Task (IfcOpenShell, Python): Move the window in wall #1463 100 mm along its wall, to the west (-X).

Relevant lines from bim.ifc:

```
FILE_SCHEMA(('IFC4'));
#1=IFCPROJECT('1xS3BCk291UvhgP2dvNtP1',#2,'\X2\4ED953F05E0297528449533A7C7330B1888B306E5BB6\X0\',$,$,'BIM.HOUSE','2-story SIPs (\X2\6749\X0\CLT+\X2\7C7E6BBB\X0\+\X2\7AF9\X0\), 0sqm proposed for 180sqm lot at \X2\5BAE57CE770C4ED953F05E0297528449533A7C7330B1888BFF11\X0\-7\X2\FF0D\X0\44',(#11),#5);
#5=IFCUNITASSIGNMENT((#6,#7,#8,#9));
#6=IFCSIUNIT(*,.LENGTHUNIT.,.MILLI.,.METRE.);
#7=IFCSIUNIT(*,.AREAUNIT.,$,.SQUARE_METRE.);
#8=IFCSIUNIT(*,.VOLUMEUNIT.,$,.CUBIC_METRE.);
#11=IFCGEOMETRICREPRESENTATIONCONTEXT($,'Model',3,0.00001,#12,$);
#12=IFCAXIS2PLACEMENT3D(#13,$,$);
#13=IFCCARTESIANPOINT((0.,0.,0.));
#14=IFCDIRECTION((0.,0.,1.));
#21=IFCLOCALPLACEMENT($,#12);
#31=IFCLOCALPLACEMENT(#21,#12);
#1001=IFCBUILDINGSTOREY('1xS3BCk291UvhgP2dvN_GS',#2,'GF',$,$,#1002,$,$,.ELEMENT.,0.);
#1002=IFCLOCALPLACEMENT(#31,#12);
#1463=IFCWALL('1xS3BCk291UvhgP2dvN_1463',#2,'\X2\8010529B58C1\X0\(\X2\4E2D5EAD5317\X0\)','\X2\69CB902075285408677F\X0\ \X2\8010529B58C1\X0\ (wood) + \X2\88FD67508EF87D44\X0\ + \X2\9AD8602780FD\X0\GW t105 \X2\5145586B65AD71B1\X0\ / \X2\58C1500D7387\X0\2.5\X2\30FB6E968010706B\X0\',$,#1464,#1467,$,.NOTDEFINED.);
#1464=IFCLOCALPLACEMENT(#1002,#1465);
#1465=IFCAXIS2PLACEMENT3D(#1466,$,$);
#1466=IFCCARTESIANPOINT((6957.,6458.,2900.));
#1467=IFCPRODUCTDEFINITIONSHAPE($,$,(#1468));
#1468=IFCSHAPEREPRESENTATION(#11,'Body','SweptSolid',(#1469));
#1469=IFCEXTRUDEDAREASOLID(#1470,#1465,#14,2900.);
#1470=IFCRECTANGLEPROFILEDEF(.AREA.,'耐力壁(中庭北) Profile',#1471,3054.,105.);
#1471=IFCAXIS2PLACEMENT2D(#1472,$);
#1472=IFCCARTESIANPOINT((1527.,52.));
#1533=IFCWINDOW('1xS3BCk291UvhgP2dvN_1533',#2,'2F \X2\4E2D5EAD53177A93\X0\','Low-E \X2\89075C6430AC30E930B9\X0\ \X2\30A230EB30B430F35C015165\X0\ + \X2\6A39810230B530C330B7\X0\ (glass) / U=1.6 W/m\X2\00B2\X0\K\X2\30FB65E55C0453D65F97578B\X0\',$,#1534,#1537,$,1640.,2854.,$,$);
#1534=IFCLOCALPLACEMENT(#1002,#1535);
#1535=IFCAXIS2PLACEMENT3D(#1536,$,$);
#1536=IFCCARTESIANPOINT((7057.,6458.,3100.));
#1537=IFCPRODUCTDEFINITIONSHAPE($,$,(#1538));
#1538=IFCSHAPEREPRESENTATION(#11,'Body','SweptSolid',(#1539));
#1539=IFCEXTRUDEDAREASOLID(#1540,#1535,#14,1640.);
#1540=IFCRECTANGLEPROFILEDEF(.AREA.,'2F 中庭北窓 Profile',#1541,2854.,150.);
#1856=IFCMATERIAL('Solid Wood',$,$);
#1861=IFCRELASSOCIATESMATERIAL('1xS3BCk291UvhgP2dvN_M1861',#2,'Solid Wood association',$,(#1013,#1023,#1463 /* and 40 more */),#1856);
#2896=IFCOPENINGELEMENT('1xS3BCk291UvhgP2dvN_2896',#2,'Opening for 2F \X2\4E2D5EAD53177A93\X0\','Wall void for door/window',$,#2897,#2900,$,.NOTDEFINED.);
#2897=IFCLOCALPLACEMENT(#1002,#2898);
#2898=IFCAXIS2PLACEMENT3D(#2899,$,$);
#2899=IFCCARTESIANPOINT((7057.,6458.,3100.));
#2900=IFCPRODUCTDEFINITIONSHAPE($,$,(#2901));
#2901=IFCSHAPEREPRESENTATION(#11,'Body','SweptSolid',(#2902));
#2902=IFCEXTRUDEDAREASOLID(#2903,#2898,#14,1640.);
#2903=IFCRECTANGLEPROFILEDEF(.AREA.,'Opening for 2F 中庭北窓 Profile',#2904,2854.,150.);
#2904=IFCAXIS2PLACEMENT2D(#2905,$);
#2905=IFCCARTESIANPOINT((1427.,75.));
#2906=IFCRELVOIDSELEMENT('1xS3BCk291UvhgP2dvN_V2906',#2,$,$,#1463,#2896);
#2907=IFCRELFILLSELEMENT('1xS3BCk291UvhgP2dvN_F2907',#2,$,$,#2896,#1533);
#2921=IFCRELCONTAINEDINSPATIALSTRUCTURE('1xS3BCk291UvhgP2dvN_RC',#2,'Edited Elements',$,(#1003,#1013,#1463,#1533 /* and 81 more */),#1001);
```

```python
import ifcopenshell
import ifcopenshell.api.geometry
import ifcopenshell.util.placement
import ifcopenshell.util.unit

model = ifcopenshell.open("bim.ifc")
unit_scale = ifcopenshell.util.unit.calculate_unit_scale(model)

window = model.by_guid("1xS3BCk291UvhgP2dvN_1533")
opening = window.FillsVoids[0].RelatingOpeningElement
wall = opening.VoidsElements[0].RelatingBuildingElement

wall_matrix = ifcopenshell.util.placement.get_local_placement(wall.ObjectPlacement)
shift = wall_matrix[:3, 0] * -0.1 / unit_scale
before = ifcopenshell.util.placement.get_local_placement(window.ObjectPlacement)[:3, 3].copy()

# The window is not placed relative to its opening, so move both.
for product in (opening, window):
    matrix = ifcopenshell.util.placement.get_local_placement(product.ObjectPlacement)
    matrix[:3, 3] += shift
    ifcopenshell.api.geometry.edit_object_placement(model, product=product, matrix=matrix, is_si=False)

after = ifcopenshell.util.placement.get_local_placement(window.ObjectPlacement)[:3, 3]
print("window moved by", (after - before).round(3) + 0.0)

model.write("bim-out.ifc")
```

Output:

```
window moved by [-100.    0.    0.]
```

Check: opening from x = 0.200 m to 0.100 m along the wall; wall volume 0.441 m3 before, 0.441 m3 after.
